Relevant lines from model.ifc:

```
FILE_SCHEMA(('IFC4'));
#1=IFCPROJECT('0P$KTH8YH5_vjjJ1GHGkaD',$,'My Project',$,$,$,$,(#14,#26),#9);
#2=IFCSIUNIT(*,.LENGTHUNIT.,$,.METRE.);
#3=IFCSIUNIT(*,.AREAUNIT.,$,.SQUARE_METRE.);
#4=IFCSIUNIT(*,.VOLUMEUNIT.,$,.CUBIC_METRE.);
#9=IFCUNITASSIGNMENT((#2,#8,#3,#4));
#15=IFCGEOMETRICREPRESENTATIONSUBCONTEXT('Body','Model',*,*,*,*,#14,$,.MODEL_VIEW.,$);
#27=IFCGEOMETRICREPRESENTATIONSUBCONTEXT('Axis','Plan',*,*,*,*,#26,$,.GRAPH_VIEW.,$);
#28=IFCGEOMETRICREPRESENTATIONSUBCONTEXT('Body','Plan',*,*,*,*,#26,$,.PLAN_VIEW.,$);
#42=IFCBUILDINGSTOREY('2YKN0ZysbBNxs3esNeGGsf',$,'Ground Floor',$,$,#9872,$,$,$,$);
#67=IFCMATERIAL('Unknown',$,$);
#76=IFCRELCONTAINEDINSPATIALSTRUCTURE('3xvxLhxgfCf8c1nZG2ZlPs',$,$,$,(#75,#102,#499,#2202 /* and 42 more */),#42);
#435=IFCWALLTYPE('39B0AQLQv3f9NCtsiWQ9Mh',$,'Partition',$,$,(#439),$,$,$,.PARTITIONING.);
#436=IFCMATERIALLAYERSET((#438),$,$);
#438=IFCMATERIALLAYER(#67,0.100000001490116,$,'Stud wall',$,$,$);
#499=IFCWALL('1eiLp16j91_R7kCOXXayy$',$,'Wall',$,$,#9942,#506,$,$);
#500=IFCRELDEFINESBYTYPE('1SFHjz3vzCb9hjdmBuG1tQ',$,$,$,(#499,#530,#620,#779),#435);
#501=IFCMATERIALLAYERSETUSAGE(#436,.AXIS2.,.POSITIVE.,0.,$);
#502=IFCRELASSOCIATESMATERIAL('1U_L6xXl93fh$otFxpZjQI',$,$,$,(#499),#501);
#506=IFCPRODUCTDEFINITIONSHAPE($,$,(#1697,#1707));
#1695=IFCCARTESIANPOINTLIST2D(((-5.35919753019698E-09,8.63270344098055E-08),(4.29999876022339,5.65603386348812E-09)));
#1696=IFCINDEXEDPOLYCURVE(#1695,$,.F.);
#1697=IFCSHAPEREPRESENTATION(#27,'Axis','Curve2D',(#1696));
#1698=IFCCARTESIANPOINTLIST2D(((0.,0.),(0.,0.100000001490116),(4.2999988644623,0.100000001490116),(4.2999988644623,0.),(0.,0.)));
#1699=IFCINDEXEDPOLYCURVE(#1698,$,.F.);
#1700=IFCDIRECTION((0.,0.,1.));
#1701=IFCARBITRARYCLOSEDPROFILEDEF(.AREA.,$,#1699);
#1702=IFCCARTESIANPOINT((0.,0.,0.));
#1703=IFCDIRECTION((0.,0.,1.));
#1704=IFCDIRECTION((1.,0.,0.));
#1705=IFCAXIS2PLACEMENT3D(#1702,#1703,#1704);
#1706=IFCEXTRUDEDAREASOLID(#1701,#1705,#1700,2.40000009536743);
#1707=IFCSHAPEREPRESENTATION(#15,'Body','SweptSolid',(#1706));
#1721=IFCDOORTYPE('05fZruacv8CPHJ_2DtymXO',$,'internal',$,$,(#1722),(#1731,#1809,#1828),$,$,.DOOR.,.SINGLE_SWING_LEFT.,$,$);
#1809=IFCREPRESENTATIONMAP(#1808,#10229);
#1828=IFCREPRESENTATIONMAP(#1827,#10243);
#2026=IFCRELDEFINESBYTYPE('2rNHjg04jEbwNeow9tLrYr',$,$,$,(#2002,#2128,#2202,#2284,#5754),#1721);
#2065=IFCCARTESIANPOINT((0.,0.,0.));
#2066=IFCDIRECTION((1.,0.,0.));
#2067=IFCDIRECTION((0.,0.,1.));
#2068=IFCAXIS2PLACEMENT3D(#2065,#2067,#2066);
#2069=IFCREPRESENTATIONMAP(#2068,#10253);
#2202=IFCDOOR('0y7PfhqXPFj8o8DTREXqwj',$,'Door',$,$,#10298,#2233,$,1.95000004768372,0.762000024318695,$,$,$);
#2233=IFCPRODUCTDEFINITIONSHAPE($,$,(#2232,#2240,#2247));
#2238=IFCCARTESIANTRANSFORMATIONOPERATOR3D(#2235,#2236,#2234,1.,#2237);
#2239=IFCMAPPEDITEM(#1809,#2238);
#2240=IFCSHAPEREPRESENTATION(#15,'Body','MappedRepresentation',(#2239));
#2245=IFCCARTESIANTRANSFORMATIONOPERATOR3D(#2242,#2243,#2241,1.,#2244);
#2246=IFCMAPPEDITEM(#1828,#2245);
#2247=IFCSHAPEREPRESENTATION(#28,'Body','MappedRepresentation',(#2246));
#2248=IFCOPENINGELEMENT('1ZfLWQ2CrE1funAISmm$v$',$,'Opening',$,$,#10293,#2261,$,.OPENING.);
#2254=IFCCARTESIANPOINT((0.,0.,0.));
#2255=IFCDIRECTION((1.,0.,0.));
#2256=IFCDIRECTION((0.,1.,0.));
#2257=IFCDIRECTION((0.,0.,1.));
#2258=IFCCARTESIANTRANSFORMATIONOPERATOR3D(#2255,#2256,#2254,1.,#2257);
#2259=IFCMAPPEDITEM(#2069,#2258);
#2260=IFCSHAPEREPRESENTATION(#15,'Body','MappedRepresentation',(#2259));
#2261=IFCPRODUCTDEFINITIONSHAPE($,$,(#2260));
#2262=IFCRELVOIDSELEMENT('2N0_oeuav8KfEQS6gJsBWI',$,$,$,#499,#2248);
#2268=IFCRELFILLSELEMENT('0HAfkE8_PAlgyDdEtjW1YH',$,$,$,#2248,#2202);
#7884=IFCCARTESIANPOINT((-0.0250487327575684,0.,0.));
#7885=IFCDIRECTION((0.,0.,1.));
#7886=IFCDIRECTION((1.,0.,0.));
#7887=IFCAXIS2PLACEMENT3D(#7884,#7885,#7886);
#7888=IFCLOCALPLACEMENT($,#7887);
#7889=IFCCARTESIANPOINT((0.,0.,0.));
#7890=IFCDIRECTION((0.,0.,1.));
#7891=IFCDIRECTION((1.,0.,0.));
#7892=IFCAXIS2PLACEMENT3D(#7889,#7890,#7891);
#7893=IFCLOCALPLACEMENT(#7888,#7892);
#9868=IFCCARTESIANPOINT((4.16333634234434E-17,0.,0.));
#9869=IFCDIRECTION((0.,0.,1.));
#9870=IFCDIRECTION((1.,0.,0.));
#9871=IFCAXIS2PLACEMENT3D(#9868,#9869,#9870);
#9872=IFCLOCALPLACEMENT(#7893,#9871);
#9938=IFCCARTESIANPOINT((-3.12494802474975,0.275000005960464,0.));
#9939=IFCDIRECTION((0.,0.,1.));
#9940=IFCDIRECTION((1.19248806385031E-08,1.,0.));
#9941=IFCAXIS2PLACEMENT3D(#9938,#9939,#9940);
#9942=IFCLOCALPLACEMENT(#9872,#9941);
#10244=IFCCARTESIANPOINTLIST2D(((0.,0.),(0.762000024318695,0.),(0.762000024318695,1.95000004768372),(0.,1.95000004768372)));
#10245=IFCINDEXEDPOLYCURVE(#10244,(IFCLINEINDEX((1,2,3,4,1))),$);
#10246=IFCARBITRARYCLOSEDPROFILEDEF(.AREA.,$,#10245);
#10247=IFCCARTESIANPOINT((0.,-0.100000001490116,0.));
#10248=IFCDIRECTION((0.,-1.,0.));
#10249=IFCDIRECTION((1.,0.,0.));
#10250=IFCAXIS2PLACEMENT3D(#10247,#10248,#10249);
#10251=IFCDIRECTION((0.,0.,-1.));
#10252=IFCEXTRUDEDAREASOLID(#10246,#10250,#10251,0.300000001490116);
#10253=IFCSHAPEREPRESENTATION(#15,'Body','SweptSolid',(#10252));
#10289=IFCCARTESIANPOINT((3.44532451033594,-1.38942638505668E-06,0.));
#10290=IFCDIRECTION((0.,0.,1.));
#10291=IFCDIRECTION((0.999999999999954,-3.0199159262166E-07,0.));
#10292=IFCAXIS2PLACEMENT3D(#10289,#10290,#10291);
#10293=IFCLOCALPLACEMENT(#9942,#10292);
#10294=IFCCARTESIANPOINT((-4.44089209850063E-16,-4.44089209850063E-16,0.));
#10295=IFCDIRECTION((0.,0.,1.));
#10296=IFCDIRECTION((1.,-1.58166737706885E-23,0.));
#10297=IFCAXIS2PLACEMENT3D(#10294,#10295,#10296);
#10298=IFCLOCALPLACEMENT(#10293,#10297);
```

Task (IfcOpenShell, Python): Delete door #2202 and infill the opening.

```python
import ifcopenshell
import ifcopenshell.api.feature
import ifcopenshell.api.root
import ifcopenshell.geom
import ifcopenshell.util.shape

model = ifcopenshell.open("model.ifc")
settings = ifcopenshell.geom.settings()


def volume(element):
    """Net volume in cubic metres, openings subtracted."""
    shape = ifcopenshell.geom.create_shape(settings, element)
    return ifcopenshell.util.shape.get_volume(shape.geometry)


door = model.by_guid("0y7PfhqXPFj8o8DTREXqwj")
opening = door.FillsVoids[0].RelatingOpeningElement
wall = opening.VoidsElements[0].RelatingBuildingElement
before = volume(wall)

ifcopenshell.api.root.remove_product(model, product=door)
ifcopenshell.api.feature.remove_feature(model, feature=opening)

after = volume(wall)

print(f"wall volume {before:.3f} -> {after:.3f} m3")

model.write("model_v2.ifc")
```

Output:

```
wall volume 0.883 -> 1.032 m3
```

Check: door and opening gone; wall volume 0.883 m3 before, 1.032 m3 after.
